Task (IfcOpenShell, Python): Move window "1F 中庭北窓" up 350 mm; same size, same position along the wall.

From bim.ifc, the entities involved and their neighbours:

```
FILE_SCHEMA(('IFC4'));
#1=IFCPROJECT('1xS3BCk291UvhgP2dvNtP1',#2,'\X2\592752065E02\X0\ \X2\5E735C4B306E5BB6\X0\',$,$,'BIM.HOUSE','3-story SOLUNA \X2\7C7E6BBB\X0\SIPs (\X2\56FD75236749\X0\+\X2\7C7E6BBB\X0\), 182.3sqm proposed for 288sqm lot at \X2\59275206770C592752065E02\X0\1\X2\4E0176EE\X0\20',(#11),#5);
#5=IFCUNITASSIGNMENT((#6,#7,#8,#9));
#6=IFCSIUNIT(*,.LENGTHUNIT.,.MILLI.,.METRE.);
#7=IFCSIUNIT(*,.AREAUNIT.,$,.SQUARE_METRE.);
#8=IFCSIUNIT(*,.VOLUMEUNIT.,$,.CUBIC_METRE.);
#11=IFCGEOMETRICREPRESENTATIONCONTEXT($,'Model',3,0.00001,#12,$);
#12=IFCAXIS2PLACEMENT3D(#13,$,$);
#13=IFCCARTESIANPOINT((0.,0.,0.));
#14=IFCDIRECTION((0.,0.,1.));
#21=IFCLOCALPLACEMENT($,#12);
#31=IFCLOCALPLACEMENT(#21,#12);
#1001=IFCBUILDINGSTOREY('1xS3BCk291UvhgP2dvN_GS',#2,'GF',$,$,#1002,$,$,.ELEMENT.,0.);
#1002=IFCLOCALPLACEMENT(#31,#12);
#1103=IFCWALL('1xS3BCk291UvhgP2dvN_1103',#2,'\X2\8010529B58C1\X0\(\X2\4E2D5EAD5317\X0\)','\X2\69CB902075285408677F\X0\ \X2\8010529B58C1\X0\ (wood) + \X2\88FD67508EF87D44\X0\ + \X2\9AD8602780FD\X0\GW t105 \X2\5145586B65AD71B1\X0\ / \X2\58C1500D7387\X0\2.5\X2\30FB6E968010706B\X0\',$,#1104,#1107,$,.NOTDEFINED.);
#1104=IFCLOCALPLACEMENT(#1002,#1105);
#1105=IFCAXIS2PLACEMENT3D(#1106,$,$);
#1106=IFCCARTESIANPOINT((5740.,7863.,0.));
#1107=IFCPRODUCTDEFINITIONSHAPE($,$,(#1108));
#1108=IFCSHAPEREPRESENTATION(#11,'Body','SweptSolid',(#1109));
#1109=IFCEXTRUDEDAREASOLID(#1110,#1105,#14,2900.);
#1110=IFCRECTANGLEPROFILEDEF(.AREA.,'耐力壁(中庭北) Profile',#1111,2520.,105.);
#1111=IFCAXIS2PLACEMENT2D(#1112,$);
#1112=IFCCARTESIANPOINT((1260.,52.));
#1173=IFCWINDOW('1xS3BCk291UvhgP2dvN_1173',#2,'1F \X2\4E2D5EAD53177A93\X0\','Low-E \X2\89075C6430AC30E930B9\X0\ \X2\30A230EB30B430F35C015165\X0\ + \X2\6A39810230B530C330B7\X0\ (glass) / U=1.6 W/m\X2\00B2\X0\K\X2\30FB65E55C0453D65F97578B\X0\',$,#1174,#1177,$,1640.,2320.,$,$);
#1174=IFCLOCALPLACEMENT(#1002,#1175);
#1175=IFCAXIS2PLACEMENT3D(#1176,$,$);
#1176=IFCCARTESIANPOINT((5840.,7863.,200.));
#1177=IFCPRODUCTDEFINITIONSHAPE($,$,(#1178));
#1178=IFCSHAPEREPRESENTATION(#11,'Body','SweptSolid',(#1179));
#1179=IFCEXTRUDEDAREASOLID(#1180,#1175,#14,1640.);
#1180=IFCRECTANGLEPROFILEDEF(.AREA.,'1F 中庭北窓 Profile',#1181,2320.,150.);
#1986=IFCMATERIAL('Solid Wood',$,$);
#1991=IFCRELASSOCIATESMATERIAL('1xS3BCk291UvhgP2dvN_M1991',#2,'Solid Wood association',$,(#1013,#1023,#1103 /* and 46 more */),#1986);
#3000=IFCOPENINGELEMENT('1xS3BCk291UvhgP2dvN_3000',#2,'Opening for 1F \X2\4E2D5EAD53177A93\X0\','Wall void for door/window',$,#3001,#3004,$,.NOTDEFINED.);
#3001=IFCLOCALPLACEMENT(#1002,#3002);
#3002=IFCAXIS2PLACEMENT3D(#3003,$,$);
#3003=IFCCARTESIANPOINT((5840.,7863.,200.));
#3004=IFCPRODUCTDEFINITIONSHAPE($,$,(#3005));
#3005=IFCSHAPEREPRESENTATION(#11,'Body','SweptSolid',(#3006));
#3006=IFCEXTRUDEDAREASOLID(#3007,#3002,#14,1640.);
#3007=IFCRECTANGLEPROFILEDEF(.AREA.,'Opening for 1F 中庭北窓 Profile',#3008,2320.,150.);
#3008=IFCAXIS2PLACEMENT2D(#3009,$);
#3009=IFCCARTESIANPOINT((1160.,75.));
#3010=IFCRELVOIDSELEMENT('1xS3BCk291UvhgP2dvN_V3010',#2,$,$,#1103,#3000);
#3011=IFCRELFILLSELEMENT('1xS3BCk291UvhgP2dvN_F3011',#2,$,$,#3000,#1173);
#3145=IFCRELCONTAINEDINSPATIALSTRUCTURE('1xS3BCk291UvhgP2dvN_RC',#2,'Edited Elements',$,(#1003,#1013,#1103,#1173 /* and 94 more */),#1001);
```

```python
import numpy as np
import ifcopenshell
import ifcopenshell.api.geometry
import ifcopenshell.util.placement
import ifcopenshell.util.unit

model = ifcopenshell.open("bim.ifc")
unit_scale = ifcopenshell.util.unit.calculate_unit_scale(model)

window = model.by_guid("1xS3BCk291UvhgP2dvN_1173")
opening = window.FillsVoids[0].RelatingOpeningElement
dz = 0.35 / unit_scale

shift = np.array([0.0, 0.0, dz])
# The window is not placed relative to its opening, so move both.
for product in (opening, window):
    matrix = ifcopenshell.util.placement.get_local_placement(product.ObjectPlacement)
    matrix[:3, 3] += shift
    ifcopenshell.api.geometry.edit_object_placement(model, product=product, matrix=matrix, is_si=False)

print(f"moved by {dz * unit_scale:+.3f} m")

model.write("bim_edited.ifc")
```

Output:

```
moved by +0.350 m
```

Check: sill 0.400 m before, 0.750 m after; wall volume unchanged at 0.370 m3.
